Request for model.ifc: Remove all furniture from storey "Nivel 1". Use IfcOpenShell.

First a look at what the model holds.

```python
import ifcopenshell
import ifcopenshell.util.element

model = ifcopenshell.open("model.ifc")
print(model.schema)
storey = next(s for s in model.by_type("IfcBuildingStorey") if s.Name == "Nivel 1")
furniture = [e for e in ifcopenshell.util.element.get_decomposition(storey) if e.is_a("IfcFurnishingElement")]
seen = {}
for e in furniture:
    element_type = ifcopenshell.util.element.get_type(e)
    name = element_type.Name if element_type not in (None, e) else None
    seen[name] = seen.get(name, 0) + 1
for name, count in sorted(seen.items(), key=str):
    print(count, "x", name)
```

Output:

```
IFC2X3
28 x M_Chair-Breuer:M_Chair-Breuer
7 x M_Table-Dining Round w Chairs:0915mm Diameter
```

```python
import ifcopenshell
import ifcopenshell.api.root
import ifcopenshell.util.element

model = ifcopenshell.open("model.ifc")

storey = next(s for s in model.by_type("IfcBuildingStorey") if s.Name == "Nivel 1")
furniture = [e for e in ifcopenshell.util.element.get_decomposition(storey) if e.is_a("IfcFurnishingElement")]

for e in furniture:
    ifcopenshell.api.root.remove_product(model, product=e)
print(len(furniture), "removed")

model.write("model_edited.ifc")
```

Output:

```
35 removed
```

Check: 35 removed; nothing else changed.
